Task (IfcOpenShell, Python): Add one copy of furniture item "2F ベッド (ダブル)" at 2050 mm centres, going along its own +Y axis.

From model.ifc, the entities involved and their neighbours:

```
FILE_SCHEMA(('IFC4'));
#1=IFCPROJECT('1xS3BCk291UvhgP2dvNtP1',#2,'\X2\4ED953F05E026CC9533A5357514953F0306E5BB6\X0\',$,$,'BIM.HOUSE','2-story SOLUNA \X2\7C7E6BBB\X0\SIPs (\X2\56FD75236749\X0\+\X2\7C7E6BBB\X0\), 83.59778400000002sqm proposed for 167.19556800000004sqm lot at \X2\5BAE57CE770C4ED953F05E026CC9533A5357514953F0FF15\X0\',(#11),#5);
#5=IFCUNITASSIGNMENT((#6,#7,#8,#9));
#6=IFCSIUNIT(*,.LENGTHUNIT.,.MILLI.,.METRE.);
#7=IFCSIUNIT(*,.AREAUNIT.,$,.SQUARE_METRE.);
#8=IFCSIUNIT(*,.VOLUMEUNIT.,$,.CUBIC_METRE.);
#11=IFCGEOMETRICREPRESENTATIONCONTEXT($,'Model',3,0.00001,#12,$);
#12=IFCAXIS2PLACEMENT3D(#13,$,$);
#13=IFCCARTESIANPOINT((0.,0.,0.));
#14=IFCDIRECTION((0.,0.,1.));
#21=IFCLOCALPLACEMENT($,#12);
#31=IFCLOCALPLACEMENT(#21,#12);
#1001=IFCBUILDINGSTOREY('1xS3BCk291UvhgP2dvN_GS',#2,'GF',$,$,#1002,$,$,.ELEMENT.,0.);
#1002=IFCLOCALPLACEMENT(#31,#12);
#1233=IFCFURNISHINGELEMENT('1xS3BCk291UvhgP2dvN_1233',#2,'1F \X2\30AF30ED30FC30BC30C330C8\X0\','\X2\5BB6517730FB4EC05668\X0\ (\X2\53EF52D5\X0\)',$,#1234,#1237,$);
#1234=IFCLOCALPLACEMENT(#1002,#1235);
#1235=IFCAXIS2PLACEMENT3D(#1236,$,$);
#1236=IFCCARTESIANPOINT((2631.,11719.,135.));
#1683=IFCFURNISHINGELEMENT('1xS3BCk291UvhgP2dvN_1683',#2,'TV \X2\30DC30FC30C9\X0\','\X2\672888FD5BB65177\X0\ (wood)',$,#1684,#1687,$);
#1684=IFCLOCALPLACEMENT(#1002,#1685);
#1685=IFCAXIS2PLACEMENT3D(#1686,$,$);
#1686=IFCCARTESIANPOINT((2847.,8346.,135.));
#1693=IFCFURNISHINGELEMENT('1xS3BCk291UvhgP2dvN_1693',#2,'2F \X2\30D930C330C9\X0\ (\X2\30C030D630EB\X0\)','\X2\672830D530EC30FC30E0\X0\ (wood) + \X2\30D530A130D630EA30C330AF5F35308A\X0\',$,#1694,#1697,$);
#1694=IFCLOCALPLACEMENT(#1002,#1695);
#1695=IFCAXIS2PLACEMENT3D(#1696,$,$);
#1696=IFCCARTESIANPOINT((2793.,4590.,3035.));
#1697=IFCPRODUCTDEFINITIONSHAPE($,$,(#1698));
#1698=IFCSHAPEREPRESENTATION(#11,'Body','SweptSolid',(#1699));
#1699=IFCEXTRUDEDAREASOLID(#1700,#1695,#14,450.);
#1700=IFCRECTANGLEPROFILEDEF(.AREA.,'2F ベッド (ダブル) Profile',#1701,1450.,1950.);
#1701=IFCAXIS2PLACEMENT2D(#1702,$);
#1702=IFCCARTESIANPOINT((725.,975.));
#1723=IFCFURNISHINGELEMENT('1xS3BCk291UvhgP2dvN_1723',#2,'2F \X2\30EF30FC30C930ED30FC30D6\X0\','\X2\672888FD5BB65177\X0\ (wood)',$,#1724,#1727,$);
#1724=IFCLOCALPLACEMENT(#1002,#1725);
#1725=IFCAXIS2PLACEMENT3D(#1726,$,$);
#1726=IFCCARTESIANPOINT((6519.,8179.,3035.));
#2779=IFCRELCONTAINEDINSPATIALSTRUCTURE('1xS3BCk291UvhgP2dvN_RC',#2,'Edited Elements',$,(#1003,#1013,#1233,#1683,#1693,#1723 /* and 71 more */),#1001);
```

```python
import ifcopenshell
import ifcopenshell.api.geometry
import ifcopenshell.api.root
import ifcopenshell.util.element
import ifcopenshell.util.placement
import ifcopenshell.util.unit

model = ifcopenshell.open("model.ifc")
unit_scale = ifcopenshell.util.unit.calculate_unit_scale(model)


def reuse_history(source, copy):
    """copy_class also copies each property set's owner history, people and application; keep the originals."""
    for rel in copy.IsDefinedBy:
        if rel.is_a("IfcRelDefinesByProperties") and (history := rel.RelatingPropertyDefinition.OwnerHistory):
            rel.RelatingPropertyDefinition.OwnerHistory = source.OwnerHistory
            ifcopenshell.util.element.remove_deep2(model, history)


source = model.by_id(1693)
base = ifcopenshell.util.placement.get_local_placement(source.ObjectPlacement)
step = base[:3, 1] * 2.05 / unit_scale

for i in range(1, 2):
    copy = ifcopenshell.api.root.copy_class(model, product=source)
    copy.Representation = ifcopenshell.util.element.copy_deep(
        model, source.Representation, exclude=["IfcGeometricRepresentationContext", "IfcRepresentationMap"]
    )
    reuse_history(source, copy)
    matrix = base.copy()
    matrix[:3, 3] += i * step
    print("added at", matrix[:3, 3].round(3) + 0.0)
    ifcopenshell.api.geometry.edit_object_placement(model, product=copy, matrix=matrix, is_si=False)

model.write("model_v2.ifc")
```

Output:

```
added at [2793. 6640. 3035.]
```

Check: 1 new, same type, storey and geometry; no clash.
